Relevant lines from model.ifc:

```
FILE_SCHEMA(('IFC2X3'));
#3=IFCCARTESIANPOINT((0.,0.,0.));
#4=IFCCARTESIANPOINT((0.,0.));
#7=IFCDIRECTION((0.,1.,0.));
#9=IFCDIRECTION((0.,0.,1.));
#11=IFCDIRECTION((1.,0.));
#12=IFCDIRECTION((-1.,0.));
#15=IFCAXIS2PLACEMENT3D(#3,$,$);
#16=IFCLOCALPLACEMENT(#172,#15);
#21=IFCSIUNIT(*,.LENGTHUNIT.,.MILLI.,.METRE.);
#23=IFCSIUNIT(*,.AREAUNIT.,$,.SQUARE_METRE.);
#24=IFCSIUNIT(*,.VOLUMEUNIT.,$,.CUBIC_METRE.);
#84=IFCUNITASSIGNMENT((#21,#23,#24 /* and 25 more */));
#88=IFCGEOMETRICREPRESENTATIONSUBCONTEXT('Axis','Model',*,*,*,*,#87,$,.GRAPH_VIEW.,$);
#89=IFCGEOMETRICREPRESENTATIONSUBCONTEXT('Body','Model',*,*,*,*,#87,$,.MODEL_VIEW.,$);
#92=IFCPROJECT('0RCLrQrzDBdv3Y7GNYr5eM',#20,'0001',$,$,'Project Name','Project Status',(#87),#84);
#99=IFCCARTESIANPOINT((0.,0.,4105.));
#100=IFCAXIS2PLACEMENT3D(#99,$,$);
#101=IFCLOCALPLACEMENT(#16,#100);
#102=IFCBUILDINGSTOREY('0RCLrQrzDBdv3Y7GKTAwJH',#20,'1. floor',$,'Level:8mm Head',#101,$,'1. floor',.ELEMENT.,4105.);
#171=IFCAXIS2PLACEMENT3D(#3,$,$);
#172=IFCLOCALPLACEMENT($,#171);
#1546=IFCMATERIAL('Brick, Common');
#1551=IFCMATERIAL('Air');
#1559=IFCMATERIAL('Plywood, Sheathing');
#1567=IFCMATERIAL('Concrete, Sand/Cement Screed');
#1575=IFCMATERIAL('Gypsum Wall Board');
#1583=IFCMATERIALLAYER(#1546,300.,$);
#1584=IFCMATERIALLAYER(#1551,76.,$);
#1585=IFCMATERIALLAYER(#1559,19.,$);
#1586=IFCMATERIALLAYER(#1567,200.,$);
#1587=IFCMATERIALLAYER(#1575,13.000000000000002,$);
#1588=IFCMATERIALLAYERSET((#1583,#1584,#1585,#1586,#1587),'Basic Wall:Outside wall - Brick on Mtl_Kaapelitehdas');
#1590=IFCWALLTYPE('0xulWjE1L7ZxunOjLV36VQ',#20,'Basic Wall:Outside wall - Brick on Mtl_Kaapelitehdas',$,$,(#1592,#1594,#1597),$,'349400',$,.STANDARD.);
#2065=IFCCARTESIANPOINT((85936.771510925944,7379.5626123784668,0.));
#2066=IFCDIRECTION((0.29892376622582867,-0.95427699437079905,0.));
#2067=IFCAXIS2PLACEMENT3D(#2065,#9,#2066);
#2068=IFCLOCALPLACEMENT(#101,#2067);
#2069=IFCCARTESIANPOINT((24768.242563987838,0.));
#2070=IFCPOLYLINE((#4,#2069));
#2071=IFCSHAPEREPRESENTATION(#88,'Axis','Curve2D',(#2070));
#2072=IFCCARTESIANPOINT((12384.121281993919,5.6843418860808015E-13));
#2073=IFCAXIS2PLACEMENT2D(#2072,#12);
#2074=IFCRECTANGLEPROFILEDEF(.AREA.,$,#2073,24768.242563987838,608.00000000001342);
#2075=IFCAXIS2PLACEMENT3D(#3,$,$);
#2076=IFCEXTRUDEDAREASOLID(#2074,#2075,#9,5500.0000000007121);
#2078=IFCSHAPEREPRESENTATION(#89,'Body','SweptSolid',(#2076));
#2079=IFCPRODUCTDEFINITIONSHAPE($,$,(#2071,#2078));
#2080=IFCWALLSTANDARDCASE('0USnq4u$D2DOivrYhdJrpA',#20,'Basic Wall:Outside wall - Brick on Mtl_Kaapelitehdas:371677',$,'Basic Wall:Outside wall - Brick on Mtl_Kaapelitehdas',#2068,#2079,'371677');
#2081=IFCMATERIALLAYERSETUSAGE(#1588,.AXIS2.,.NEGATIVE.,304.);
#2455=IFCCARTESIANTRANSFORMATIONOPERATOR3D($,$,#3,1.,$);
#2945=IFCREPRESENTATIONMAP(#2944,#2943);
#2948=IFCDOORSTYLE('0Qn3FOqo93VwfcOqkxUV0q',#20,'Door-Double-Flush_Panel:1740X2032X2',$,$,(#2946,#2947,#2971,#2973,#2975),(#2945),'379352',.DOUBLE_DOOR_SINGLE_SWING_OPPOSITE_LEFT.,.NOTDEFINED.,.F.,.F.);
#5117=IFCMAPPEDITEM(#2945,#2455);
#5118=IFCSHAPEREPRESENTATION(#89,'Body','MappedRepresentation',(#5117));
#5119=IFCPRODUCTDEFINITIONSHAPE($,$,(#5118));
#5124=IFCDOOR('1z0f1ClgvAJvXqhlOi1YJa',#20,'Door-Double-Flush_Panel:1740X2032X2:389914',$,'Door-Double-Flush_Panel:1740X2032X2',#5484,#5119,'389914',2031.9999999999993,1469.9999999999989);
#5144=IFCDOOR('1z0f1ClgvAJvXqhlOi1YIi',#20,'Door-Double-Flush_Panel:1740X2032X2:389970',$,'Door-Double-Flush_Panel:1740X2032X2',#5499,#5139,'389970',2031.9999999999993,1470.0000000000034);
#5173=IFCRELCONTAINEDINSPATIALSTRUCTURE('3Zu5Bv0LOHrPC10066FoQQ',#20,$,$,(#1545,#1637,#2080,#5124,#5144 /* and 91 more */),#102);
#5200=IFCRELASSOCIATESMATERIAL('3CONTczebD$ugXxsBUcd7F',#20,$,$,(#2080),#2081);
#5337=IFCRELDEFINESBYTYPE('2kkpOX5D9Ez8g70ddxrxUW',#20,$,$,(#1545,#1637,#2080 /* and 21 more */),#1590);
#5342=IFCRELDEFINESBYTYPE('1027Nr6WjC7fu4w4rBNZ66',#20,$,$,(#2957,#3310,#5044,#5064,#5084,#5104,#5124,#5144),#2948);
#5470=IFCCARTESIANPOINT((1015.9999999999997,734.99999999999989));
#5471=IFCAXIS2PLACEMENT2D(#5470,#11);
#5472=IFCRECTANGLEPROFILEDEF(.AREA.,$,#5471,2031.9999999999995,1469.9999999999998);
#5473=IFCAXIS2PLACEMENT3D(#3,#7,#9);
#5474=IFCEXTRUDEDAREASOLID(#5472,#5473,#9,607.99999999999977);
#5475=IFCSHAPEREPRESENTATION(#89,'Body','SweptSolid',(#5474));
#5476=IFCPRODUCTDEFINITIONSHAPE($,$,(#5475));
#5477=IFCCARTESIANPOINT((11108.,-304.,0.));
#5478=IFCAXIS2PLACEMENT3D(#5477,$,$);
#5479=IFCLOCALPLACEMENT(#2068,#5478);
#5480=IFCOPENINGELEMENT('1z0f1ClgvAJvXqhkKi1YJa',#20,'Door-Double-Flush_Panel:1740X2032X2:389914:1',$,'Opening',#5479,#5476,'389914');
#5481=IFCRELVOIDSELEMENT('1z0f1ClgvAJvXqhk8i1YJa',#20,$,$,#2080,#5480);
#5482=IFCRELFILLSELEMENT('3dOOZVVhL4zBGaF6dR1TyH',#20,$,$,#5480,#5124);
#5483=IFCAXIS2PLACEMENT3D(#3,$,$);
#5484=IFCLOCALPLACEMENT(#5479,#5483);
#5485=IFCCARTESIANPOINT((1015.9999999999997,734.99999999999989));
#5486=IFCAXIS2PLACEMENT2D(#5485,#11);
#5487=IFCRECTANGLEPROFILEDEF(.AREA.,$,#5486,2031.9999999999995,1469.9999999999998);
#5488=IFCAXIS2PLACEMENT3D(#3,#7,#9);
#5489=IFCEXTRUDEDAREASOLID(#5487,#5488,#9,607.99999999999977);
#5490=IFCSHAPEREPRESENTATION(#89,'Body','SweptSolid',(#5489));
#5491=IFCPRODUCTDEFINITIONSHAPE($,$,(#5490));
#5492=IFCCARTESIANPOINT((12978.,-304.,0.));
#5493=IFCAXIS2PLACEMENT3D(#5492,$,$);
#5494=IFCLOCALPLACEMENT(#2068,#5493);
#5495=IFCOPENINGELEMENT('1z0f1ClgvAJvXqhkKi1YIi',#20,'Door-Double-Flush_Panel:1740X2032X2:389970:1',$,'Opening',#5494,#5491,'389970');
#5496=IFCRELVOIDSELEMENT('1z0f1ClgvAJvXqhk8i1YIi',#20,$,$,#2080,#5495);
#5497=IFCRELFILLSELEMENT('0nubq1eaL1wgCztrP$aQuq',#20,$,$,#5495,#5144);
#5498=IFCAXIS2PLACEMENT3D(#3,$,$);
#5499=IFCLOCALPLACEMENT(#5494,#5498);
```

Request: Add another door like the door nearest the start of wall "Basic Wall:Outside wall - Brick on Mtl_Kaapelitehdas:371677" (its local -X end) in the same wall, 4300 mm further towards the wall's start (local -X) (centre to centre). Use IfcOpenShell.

```python
import ifcopenshell
import ifcopenshell.api.feature
import ifcopenshell.api.geometry
import ifcopenshell.api.root
import ifcopenshell.geom
import ifcopenshell.util.element
import ifcopenshell.util.placement
import ifcopenshell.util.shape
import ifcopenshell.util.unit

model = ifcopenshell.open("model.ifc")
unit_scale = ifcopenshell.util.unit.calculate_unit_scale(model)
settings = ifcopenshell.geom.settings()


def volume(element):
    """Net volume in cubic metres, openings subtracted."""
    shape = ifcopenshell.geom.create_shape(settings, element)
    return ifcopenshell.util.shape.get_volume(shape.geometry)


def reuse_history(source, copy):
    """copy_class also copies each property set's owner history, people and application; keep the originals."""
    for rel in copy.IsDefinedBy:
        if rel.is_a("IfcRelDefinesByProperties") and (history := rel.RelatingPropertyDefinition.OwnerHistory):
            rel.RelatingPropertyDefinition.OwnerHistory = source.OwnerHistory
            ifcopenshell.util.element.remove_deep2(model, history)


door = model.by_guid("1z0f1ClgvAJvXqhlOi1YJa")
opening = door.FillsVoids[0].RelatingOpeningElement
wall = opening.VoidsElements[0].RelatingBuildingElement
before = volume(wall)
shift = ifcopenshell.util.placement.get_local_placement(wall.ObjectPlacement)[:3, 0] * -4.3 / unit_scale

# copy_class copies the void relationship, type, container and properties, but no geometry.
new_opening = ifcopenshell.api.root.copy_class(model, product=opening)
new_opening.Representation = ifcopenshell.util.element.copy_deep(
    model, opening.Representation, exclude=["IfcGeometricRepresentationContext", "IfcRepresentationMap"]
)
new_opening.Name = "Door-Double-Flush_Panel:1740X2032X2"
new_opening.Tag = None
new_door = ifcopenshell.api.root.copy_class(model, product=door)
new_door.Representation = ifcopenshell.util.element.copy_deep(
    model, door.Representation, exclude=["IfcGeometricRepresentationContext", "IfcRepresentationMap"]
)
new_door.Name = "Door-Double-Flush_Panel:1740X2032X2"
new_door.Tag = None
reuse_history(door, new_door)
fills = ifcopenshell.api.feature.add_filling(model, opening=new_opening, element=new_door)
fills.OwnerHistory = new_door.OwnerHistory  # required in IFC2X3

for old, new in ((opening, new_opening), (door, new_door)):
    matrix = ifcopenshell.util.placement.get_local_placement(old.ObjectPlacement)
    matrix[:3, 3] += shift
    ifcopenshell.api.geometry.edit_object_placement(model, product=new, matrix=matrix, is_si=False)

after = volume(wall)

print(f"wall volume {before:.3f} -> {after:.3f} m3")

model.write("model_edited.ifc")
```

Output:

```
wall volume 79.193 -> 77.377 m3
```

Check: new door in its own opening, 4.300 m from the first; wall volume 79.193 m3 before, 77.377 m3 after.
